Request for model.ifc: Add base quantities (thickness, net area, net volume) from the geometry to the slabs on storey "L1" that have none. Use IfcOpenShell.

First a look at what the model holds.

```python
import ifcopenshell
import ifcopenshell.util.element
import ifcopenshell.util.unit

model = ifcopenshell.open("model.ifc")
print(model.schema)
for unit_type in ("LENGTHUNIT", "AREAUNIT", "VOLUMEUNIT"):
    print(unit_type, ifcopenshell.util.unit.calculate_unit_scale(model, unit_type))
storey = next(s for s in model.by_type("IfcBuildingStorey") if s.Name == "L1")
slabs = [e for e in ifcopenshell.util.element.get_decomposition(storey) if e.is_a("IfcSlab")]
for e in sorted(slabs, key=lambda e: e.id()):
    print(e.id(), e.is_a(), e.Name, list(ifcopenshell.util.element.get_psets(e, qtos_only=True)), sep=" | ")
```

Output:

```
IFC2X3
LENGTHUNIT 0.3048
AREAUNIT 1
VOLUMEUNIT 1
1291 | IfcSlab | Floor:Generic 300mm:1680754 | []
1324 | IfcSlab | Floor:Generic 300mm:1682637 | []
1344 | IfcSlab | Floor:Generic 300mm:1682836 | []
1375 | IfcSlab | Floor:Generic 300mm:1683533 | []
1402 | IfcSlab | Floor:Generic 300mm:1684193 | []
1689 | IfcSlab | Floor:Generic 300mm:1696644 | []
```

```python
import ifcopenshell
import ifcopenshell.api.pset
import ifcopenshell.geom
import ifcopenshell.util.element
import ifcopenshell.util.shape
import ifcopenshell.util.unit

model = ifcopenshell.open("model.ifc")
unit_scale = ifcopenshell.util.unit.calculate_unit_scale(model)
area_scale = ifcopenshell.util.unit.calculate_unit_scale(model, "AREAUNIT")
volume_scale = ifcopenshell.util.unit.calculate_unit_scale(model, "VOLUMEUNIT")
settings = ifcopenshell.geom.settings()

storey = next(s for s in model.by_type("IfcBuildingStorey") if s.Name == "L1")
slabs = [e for e in ifcopenshell.util.element.get_decomposition(storey) if e.is_a("IfcSlab")]

for e in sorted(slabs, key=lambda e: e.id()):
    if ifcopenshell.util.element.get_psets(e, qtos_only=True, should_inherit=False):
        continue
    # Geometry comes back in metres, in the element's own axes.
    shape = ifcopenshell.geom.create_shape(settings, e)
    values = {
        "Width": ifcopenshell.util.shape.get_z(shape.geometry) / unit_scale,
        "NetArea": ifcopenshell.util.shape.get_footprint_area(shape.geometry) / area_scale,
        "NetVolume": ifcopenshell.util.shape.get_volume(shape.geometry) / volume_scale,
    }
    qto = ifcopenshell.api.pset.add_qto(model, product=e, name="BaseQuantities")
    ifcopenshell.api.pset.edit_qto(model, qto=qto, properties=values)
    print(e.id(), {k: round(v, 3) for k, v in values.items()})

model.write("model_v2.ifc")
```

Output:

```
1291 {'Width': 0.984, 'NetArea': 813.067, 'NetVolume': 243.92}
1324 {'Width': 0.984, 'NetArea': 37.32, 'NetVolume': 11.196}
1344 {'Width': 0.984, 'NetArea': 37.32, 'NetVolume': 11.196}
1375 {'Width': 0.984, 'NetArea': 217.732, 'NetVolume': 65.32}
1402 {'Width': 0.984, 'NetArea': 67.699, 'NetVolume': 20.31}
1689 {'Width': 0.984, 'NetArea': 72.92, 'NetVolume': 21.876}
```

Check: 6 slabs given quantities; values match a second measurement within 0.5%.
